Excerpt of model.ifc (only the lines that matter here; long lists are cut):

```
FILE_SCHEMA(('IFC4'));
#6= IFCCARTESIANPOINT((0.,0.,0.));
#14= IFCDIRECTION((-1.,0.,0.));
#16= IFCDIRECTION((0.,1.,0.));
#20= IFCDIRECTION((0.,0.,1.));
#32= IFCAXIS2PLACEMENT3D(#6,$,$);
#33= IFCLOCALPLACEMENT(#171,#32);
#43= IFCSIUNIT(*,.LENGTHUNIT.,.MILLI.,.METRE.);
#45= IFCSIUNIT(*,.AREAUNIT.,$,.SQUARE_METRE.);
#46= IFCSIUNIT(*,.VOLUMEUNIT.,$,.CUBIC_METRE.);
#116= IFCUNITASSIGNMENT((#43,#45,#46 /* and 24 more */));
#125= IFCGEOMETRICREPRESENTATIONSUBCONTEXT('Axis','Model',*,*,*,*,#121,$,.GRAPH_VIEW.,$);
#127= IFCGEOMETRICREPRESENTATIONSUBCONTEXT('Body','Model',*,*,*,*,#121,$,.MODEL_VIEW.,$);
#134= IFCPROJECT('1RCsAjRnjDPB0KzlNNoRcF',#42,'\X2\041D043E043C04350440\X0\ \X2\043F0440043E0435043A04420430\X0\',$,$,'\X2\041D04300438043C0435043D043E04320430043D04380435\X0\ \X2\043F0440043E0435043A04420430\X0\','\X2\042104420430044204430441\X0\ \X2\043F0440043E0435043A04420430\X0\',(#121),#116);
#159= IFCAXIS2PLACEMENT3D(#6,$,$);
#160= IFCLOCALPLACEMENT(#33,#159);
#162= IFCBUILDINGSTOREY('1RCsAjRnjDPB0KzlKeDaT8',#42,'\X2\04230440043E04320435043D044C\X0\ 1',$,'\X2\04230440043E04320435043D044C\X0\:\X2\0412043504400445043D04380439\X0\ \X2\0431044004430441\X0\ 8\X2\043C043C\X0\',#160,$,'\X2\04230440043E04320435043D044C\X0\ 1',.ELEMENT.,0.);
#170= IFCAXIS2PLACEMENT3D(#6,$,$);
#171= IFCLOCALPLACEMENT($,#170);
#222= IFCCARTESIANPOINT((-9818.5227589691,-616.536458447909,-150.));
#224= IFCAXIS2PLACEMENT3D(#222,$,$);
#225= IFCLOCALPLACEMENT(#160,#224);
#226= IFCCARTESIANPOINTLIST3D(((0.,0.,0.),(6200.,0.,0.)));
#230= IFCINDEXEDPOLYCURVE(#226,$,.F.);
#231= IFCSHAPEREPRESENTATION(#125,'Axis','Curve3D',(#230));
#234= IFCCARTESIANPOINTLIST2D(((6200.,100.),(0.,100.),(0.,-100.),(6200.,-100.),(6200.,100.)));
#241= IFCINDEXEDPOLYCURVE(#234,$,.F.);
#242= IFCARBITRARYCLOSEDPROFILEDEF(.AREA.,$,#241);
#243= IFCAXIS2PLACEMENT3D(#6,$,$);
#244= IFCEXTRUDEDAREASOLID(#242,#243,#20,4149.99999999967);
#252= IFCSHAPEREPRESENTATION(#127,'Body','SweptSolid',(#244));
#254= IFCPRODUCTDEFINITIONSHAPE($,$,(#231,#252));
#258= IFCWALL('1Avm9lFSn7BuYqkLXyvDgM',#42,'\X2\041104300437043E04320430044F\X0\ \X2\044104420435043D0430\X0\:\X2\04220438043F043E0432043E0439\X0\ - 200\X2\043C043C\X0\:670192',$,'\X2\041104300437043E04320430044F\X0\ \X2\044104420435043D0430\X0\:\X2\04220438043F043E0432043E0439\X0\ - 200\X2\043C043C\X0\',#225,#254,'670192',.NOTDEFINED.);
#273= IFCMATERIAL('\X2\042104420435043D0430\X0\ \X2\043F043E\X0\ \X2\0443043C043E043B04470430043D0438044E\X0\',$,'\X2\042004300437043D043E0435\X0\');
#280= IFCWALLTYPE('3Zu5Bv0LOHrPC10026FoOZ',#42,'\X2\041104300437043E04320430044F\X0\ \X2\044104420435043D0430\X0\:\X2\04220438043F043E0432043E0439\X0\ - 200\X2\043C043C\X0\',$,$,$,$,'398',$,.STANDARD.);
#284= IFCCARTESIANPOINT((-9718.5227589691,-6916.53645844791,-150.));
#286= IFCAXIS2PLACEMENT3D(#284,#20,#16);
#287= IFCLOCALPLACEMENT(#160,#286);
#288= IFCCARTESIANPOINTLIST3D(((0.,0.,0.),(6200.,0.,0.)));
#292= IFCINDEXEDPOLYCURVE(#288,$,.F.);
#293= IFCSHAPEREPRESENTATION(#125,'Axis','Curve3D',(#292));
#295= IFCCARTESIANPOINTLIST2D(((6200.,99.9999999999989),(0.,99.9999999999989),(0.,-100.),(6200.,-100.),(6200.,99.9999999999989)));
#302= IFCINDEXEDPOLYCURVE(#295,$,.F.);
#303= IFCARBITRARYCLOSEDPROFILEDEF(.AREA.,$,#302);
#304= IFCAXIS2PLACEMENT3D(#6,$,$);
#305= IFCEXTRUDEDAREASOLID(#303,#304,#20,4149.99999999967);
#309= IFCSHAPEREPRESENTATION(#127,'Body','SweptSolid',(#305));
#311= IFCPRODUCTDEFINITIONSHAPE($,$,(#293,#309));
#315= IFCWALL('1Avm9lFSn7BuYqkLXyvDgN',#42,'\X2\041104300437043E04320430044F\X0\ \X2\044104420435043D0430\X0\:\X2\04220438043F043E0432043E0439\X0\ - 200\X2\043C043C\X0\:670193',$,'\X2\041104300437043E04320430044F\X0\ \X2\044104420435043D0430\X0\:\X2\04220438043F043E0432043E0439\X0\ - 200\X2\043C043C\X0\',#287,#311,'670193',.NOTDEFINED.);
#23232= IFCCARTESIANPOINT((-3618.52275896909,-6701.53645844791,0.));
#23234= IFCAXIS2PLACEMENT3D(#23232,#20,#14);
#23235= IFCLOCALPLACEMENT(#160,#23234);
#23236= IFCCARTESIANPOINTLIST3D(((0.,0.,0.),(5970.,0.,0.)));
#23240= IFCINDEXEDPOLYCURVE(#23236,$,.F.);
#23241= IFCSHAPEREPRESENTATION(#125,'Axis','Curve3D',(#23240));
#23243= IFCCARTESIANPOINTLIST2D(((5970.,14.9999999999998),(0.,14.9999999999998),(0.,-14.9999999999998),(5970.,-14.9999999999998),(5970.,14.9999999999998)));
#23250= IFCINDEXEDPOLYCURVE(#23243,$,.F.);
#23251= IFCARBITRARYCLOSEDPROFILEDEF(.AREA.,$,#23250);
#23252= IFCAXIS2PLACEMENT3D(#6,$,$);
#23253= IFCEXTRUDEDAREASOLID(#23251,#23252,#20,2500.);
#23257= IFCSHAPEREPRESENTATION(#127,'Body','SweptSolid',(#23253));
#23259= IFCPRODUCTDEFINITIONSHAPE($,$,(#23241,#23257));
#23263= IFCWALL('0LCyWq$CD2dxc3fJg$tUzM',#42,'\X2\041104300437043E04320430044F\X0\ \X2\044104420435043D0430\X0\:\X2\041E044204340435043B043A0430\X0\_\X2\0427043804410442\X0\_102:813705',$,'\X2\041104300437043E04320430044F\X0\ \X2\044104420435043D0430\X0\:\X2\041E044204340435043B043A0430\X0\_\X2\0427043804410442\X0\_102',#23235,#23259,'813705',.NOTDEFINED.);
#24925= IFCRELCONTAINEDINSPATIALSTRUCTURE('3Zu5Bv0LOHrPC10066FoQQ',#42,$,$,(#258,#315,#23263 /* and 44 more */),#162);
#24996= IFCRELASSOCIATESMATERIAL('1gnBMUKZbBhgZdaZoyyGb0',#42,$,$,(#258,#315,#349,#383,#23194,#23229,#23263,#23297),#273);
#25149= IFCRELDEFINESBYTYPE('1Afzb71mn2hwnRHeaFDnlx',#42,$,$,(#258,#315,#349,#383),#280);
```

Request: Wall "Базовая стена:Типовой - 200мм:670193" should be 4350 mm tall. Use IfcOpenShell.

```python
import ifcopenshell
import ifcopenshell.geom
import ifcopenshell.util.representation
import ifcopenshell.util.shape
import ifcopenshell.util.unit

model = ifcopenshell.open("model.ifc")
unit_scale = ifcopenshell.util.unit.calculate_unit_scale(model)
settings = ifcopenshell.geom.settings()


def volume(element):
    """Net volume in cubic metres, openings subtracted."""
    shape = ifcopenshell.geom.create_shape(settings, element)
    return ifcopenshell.util.shape.get_volume(shape.geometry)


wall = model.by_id(315)
before = volume(wall)

body = ifcopenshell.util.representation.get_representation(wall, "Model", "Body")
solid = body.Items[0]
old_height = solid.Depth
solid.Depth = 4.35 / unit_scale
after = volume(wall)

print(f"height {old_height:g} -> {solid.Depth:g}, volume {before:.3f} -> {after:.3f} m3")

model.write("model-out.ifc")
```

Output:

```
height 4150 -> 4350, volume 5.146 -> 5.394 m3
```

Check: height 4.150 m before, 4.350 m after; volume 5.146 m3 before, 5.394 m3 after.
